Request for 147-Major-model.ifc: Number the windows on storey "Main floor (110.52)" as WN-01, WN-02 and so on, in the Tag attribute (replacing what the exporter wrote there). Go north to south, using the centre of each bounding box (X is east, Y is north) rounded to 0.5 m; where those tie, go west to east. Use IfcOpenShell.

First a look at what the model holds.

```python
import ifcopenshell
import ifcopenshell.util.element
import ifcopenshell.util.placement

model = ifcopenshell.open("147-Major-model.ifc")
print(model.schema)
storey = next(s for s in model.by_type("IfcBuildingStorey") if s.Name == "Main floor (110.52)")
windows = [e for e in ifcopenshell.util.element.get_decomposition(storey) if e.is_a("IfcWindow")]
for e in sorted(windows, key=lambda e: e.id()):
    origin = ifcopenshell.util.placement.get_local_placement(e.ObjectPlacement)[:3, 3]
    print(e.id(), e.Tag, e.Name, origin.round(2) + 0.0, sep=" | ")
```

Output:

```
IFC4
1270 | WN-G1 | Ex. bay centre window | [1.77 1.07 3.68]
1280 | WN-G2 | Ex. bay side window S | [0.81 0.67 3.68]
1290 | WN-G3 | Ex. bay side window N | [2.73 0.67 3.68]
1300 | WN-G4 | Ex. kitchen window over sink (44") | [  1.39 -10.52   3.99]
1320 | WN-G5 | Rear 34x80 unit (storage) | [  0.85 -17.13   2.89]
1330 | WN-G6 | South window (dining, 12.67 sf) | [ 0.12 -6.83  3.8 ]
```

```python
import ifcopenshell
import ifcopenshell.geom
import ifcopenshell.util.element
import ifcopenshell.util.shape

model = ifcopenshell.open("147-Major-model.ifc")
settings = ifcopenshell.geom.settings()
settings.set("use-world-coords", True)


def centre(element):
    shape = ifcopenshell.geom.create_shape(settings, element)
    return ifcopenshell.util.shape.get_bbox_centroid(shape.geometry)


storey = next(s for s in model.by_type("IfcBuildingStorey") if s.Name == "Main floor (110.52)")
windows = [e for e in ifcopenshell.util.element.get_decomposition(storey) if e.is_a("IfcWindow")]

# Insertion points can sit at a corner or the storey origin, so sort by the geometry (in metres).
centres = {e: centre(e) for e in windows}
windows.sort(key=lambda e: (-round(centres[e][1] / 0.5), centres[e][0]))

for i, e in enumerate(windows, start=1):
    number = f"WN-{i:02d}"
    e.Tag = number
    print(e.id(), number)

model.write("147-Major-model_v2.ifc")
```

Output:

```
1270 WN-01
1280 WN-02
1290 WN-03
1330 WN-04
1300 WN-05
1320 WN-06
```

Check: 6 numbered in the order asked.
